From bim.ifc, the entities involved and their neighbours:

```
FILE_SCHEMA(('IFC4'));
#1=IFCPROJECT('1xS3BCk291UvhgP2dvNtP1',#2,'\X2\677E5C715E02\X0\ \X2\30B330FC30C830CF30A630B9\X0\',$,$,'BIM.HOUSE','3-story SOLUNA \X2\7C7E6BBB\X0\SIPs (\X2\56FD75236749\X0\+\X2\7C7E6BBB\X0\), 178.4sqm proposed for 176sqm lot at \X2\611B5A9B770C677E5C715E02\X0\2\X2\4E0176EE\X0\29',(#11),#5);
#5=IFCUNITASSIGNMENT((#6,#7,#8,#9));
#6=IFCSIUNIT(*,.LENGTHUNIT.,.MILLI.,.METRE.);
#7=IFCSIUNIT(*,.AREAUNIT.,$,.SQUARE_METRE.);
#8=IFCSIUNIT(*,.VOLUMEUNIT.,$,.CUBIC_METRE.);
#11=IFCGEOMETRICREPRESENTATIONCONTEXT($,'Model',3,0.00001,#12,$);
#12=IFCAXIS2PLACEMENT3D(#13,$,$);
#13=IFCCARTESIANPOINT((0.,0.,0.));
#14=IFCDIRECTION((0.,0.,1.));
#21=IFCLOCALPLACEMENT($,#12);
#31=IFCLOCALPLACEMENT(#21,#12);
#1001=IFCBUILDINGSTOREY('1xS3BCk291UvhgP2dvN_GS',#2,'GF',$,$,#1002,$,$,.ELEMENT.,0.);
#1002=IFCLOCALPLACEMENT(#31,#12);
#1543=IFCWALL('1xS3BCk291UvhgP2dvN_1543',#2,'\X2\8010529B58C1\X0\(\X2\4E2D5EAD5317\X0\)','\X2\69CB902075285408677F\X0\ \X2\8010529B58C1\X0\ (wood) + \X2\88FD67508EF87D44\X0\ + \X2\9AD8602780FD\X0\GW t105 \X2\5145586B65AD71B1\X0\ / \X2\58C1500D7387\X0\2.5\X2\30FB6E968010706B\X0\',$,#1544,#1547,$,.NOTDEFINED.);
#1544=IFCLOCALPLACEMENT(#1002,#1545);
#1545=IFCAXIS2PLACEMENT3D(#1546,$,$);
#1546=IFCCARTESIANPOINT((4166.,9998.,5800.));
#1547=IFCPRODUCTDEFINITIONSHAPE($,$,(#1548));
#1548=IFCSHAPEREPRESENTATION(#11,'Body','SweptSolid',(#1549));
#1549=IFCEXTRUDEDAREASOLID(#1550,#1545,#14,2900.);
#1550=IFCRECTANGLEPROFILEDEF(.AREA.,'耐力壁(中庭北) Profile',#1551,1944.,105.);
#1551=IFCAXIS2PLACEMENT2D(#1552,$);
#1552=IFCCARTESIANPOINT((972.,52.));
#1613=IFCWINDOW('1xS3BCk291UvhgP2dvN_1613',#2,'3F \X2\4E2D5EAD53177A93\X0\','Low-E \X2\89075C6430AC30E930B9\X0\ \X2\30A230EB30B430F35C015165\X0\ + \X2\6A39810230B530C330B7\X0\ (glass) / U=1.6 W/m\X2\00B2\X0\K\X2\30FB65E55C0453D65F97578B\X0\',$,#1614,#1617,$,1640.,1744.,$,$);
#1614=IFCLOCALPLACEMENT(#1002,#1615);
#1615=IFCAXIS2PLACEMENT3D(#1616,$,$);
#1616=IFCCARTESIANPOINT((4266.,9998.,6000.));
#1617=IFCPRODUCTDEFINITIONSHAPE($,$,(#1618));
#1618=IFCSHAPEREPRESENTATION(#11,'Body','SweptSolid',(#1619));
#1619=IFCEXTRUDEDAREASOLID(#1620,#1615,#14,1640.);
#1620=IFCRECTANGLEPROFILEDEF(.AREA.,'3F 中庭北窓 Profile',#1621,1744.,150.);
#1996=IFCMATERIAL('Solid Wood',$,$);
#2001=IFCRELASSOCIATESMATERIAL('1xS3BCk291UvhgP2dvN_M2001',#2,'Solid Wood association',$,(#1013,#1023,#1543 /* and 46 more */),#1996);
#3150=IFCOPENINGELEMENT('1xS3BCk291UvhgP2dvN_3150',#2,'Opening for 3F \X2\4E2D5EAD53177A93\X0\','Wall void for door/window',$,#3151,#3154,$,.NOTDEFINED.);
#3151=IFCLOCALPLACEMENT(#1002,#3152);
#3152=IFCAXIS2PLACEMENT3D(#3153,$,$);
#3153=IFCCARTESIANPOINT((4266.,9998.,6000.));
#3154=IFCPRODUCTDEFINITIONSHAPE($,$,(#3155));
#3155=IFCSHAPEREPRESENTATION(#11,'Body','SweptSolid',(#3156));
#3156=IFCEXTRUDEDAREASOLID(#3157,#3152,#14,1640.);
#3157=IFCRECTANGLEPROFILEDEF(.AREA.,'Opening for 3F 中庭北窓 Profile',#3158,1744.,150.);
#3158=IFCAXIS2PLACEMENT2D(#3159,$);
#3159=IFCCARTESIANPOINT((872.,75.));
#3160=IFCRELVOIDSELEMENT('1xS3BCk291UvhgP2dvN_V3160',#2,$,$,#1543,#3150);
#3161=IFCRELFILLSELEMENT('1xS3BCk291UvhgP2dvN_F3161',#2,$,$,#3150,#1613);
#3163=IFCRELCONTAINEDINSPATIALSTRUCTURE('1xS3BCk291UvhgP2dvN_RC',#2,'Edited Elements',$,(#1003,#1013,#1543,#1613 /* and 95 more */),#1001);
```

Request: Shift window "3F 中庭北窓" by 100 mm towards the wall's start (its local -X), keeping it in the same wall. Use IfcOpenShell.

```python
import ifcopenshell
import ifcopenshell.api.geometry
import ifcopenshell.util.placement
import ifcopenshell.util.unit

model = ifcopenshell.open("bim.ifc")
unit_scale = ifcopenshell.util.unit.calculate_unit_scale(model)

window = model.by_guid("1xS3BCk291UvhgP2dvN_1613")
opening = window.FillsVoids[0].RelatingOpeningElement
wall = opening.VoidsElements[0].RelatingBuildingElement

wall_matrix = ifcopenshell.util.placement.get_local_placement(wall.ObjectPlacement)
shift = wall_matrix[:3, 0] * -0.1 / unit_scale
before = ifcopenshell.util.placement.get_local_placement(window.ObjectPlacement)[:3, 3].copy()

# The window is not placed relative to its opening, so move both.
for product in (opening, window):
    matrix = ifcopenshell.util.placement.get_local_placement(product.ObjectPlacement)
    matrix[:3, 3] += shift
    ifcopenshell.api.geometry.edit_object_placement(model, product=product, matrix=matrix, is_si=False)

after = ifcopenshell.util.placement.get_local_placement(window.ObjectPlacement)[:3, 3]
print("window moved by", (after - before).round(3) + 0.0)

model.write("bim_v2.ifc")
```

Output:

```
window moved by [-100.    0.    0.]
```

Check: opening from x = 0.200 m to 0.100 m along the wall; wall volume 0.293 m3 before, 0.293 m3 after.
